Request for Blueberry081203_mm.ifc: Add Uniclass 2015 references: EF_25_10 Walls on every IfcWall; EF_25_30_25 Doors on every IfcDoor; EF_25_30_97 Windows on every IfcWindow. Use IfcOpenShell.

First a look at what the model holds.

```python
import ifcopenshell

model = ifcopenshell.open("Blueberry081203_mm.ifc")
print(model.schema)
print("classifications:", [c.Name for c in model.by_type("IfcClassification")])
for ifc_class in ("IfcDoor", "IfcRoof", "IfcStair", "IfcWall", "IfcWindow"):
    print(ifc_class, len(model.by_type(ifc_class)))
```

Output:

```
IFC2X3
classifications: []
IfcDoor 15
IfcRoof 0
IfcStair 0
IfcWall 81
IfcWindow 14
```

```python
import ifcopenshell
import ifcopenshell.api.classification

model = ifcopenshell.open("Blueberry081203_mm.ifc")

# IFC2X3 requires Source and Edition and has no link from the project to the system.
system = model.create_entity("IfcClassification", Source="NBS", Edition="2015", Name="Uniclass 2015")

codes = {
    "IfcWall": ("EF_25_10", "Walls"),
    "IfcDoor": ("EF_25_30_25", "Doors"),
    "IfcWindow": ("EF_25_30_97", "Windows"),
}
for ifc_class, (code, name) in codes.items():
    products = model.by_type(ifc_class)
    ifcopenshell.api.classification.add_reference(
        model, products=products, classification=system, identification=code, name=name
    )
    print(code, len(products))

model.write("Blueberry081203_mm_updated.ifc")
```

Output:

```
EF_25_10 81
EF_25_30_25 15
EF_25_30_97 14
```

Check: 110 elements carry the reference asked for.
